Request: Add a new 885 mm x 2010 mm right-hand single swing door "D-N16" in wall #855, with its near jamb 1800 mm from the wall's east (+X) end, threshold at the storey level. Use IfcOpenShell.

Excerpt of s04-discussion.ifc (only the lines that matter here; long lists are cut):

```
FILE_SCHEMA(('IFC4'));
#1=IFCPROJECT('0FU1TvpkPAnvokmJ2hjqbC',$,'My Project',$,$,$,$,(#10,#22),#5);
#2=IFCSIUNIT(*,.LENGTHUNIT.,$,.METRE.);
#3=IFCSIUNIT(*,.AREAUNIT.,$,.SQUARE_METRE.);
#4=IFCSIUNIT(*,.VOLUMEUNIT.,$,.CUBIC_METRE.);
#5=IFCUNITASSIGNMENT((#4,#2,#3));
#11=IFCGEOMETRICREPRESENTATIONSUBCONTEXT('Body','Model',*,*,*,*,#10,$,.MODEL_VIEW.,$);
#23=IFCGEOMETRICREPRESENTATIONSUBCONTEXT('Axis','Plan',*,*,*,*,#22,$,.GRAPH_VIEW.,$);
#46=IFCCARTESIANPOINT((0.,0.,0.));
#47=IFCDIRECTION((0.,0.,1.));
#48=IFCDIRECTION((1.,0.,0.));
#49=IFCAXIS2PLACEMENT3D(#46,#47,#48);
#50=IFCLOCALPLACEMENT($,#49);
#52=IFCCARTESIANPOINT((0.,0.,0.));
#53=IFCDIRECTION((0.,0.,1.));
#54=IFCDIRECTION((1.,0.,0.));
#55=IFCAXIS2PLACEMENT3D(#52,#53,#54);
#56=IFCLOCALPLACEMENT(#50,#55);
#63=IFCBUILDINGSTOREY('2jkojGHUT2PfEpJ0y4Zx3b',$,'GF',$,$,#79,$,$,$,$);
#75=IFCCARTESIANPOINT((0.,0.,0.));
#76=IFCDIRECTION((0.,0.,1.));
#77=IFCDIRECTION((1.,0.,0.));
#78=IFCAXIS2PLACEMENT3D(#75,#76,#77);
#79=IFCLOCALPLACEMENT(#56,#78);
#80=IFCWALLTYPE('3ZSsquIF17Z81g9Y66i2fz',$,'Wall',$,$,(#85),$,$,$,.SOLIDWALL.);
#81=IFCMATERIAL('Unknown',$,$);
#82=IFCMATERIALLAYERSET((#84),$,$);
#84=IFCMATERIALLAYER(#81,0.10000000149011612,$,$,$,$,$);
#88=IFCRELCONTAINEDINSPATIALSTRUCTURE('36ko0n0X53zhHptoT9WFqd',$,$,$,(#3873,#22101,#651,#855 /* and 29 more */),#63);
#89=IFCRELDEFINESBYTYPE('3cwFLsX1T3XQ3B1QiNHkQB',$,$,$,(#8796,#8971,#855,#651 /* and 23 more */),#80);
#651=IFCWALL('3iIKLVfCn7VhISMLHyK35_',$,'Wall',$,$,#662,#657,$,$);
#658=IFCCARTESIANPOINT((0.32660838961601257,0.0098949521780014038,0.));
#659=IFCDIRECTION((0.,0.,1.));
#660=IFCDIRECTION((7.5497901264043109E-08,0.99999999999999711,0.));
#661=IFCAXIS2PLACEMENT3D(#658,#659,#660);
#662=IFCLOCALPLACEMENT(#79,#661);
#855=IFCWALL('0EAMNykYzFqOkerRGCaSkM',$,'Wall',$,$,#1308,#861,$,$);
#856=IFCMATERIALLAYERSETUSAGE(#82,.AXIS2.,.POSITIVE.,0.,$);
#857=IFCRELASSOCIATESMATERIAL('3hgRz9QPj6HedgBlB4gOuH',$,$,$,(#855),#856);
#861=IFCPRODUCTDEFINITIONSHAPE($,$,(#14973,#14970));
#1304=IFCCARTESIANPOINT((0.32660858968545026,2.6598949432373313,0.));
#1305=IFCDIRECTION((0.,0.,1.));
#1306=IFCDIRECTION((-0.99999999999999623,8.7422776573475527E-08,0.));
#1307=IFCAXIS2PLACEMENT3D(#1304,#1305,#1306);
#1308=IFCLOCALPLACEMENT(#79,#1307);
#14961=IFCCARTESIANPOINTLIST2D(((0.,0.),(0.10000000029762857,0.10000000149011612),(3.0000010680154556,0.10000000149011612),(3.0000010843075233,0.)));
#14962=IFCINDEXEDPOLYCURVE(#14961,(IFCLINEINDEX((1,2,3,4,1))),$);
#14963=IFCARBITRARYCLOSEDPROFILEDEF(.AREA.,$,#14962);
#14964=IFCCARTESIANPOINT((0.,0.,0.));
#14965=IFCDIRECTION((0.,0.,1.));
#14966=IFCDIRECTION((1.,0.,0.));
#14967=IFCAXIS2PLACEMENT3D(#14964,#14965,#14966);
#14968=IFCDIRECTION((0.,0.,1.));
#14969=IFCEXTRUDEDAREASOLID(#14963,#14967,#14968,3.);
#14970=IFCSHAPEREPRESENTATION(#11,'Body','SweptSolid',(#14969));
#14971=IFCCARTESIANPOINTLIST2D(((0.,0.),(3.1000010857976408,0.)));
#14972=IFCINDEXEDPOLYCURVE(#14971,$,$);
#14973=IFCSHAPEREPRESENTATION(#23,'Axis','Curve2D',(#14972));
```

```python
import numpy as np
import ifcopenshell
import ifcopenshell.api.feature
import ifcopenshell.api.geometry
import ifcopenshell.api.root
import ifcopenshell.api.spatial
import ifcopenshell.geom
import ifcopenshell.util.element
import ifcopenshell.util.placement
import ifcopenshell.util.representation
import ifcopenshell.util.shape
import ifcopenshell.util.unit

model = ifcopenshell.open("s04-discussion.ifc")
unit_scale = ifcopenshell.util.unit.calculate_unit_scale(model)
settings = ifcopenshell.geom.settings()


def volume(element):
    """Net volume in cubic metres, openings subtracted."""
    shape = ifcopenshell.geom.create_shape(settings, element)
    return ifcopenshell.util.shape.get_volume(shape.geometry)


wall = model.by_id(855)
storey = ifcopenshell.util.element.get_container(wall, ifc_class="IfcBuildingStorey")
context = ifcopenshell.util.representation.get_context(model, "Model", "Body", "MODEL_VIEW")
before = volume(wall)

width, height, from_end, sill = 0.885, 2.01, 1.8, 0.0  # metres

# The wall runs along its own X axis, and the end named is its -X end.
wall_shape = ifcopenshell.geom.create_shape(settings, wall)
x, y, z = ifcopenshell.util.shape.get_vertices(wall_shape.geometry).T
start = x.min() + from_end
face, thickness = float(y.min()), float(y.max() - y.min())
wall_matrix = ifcopenshell.util.placement.get_local_placement(wall.ObjectPlacement)
level = ifcopenshell.util.placement.get_local_placement(storey.ObjectPlacement)[2, 3]


def in_wall(x, y):
    """Placement at x, y metres in the wall's axes, at sill height."""
    matrix = wall_matrix.copy()
    matrix[:, 3] = wall_matrix @ np.array([x / unit_scale, y / unit_scale, 0.0, 1.0])
    matrix[2, 3] = level + sill / unit_scale
    return matrix


# Opening: a box that overshoots both wall faces by 50 mm.
opening = ifcopenshell.api.root.create_entity(model, ifc_class="IfcOpeningElement", predefined_type="OPENING")
box = ifcopenshell.api.geometry.add_wall_representation(
    model, context=context, length=width, height=height, thickness=thickness + 0.1
)
ifcopenshell.api.geometry.assign_representation(model, product=opening, representation=box)
ifcopenshell.api.geometry.edit_object_placement(model, product=opening, matrix=in_wall(start, face - 0.05), is_si=False)
ifcopenshell.api.feature.add_feature(model, feature=opening, element=wall)

door = ifcopenshell.api.root.create_entity(model, ifc_class="IfcDoor", name="D-N16", predefined_type="DOOR")
door.OverallWidth, door.OverallHeight = width / unit_scale, height / unit_scale
door.OperationType = "SINGLE_SWING_RIGHT"
body = ifcopenshell.api.geometry.add_door_representation(
    model,
    context=context,
    overall_width=door.OverallWidth,
    overall_height=door.OverallHeight,
    operation_type="SINGLE_SWING_RIGHT",
    lining_properties={"LiningDepth": thickness / unit_scale, "ThresholdDepth": thickness / unit_scale},
)
ifcopenshell.api.geometry.assign_representation(model, product=door, representation=body)
ifcopenshell.api.spatial.assign_container(model, products=[door], relating_structure=storey)
ifcopenshell.api.feature.add_filling(model, opening=opening, element=door)

# The lining spans the wall, so the door starts at the wall face.
ifcopenshell.api.geometry.edit_object_placement(model, product=door, matrix=in_wall(start, face), is_si=False)

after = volume(wall)

print(f"wall volume {before:.3f} -> {after:.3f} m3")

model.write("s04-discussion-out.ifc")
```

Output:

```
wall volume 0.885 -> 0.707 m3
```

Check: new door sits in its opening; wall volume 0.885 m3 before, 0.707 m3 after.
